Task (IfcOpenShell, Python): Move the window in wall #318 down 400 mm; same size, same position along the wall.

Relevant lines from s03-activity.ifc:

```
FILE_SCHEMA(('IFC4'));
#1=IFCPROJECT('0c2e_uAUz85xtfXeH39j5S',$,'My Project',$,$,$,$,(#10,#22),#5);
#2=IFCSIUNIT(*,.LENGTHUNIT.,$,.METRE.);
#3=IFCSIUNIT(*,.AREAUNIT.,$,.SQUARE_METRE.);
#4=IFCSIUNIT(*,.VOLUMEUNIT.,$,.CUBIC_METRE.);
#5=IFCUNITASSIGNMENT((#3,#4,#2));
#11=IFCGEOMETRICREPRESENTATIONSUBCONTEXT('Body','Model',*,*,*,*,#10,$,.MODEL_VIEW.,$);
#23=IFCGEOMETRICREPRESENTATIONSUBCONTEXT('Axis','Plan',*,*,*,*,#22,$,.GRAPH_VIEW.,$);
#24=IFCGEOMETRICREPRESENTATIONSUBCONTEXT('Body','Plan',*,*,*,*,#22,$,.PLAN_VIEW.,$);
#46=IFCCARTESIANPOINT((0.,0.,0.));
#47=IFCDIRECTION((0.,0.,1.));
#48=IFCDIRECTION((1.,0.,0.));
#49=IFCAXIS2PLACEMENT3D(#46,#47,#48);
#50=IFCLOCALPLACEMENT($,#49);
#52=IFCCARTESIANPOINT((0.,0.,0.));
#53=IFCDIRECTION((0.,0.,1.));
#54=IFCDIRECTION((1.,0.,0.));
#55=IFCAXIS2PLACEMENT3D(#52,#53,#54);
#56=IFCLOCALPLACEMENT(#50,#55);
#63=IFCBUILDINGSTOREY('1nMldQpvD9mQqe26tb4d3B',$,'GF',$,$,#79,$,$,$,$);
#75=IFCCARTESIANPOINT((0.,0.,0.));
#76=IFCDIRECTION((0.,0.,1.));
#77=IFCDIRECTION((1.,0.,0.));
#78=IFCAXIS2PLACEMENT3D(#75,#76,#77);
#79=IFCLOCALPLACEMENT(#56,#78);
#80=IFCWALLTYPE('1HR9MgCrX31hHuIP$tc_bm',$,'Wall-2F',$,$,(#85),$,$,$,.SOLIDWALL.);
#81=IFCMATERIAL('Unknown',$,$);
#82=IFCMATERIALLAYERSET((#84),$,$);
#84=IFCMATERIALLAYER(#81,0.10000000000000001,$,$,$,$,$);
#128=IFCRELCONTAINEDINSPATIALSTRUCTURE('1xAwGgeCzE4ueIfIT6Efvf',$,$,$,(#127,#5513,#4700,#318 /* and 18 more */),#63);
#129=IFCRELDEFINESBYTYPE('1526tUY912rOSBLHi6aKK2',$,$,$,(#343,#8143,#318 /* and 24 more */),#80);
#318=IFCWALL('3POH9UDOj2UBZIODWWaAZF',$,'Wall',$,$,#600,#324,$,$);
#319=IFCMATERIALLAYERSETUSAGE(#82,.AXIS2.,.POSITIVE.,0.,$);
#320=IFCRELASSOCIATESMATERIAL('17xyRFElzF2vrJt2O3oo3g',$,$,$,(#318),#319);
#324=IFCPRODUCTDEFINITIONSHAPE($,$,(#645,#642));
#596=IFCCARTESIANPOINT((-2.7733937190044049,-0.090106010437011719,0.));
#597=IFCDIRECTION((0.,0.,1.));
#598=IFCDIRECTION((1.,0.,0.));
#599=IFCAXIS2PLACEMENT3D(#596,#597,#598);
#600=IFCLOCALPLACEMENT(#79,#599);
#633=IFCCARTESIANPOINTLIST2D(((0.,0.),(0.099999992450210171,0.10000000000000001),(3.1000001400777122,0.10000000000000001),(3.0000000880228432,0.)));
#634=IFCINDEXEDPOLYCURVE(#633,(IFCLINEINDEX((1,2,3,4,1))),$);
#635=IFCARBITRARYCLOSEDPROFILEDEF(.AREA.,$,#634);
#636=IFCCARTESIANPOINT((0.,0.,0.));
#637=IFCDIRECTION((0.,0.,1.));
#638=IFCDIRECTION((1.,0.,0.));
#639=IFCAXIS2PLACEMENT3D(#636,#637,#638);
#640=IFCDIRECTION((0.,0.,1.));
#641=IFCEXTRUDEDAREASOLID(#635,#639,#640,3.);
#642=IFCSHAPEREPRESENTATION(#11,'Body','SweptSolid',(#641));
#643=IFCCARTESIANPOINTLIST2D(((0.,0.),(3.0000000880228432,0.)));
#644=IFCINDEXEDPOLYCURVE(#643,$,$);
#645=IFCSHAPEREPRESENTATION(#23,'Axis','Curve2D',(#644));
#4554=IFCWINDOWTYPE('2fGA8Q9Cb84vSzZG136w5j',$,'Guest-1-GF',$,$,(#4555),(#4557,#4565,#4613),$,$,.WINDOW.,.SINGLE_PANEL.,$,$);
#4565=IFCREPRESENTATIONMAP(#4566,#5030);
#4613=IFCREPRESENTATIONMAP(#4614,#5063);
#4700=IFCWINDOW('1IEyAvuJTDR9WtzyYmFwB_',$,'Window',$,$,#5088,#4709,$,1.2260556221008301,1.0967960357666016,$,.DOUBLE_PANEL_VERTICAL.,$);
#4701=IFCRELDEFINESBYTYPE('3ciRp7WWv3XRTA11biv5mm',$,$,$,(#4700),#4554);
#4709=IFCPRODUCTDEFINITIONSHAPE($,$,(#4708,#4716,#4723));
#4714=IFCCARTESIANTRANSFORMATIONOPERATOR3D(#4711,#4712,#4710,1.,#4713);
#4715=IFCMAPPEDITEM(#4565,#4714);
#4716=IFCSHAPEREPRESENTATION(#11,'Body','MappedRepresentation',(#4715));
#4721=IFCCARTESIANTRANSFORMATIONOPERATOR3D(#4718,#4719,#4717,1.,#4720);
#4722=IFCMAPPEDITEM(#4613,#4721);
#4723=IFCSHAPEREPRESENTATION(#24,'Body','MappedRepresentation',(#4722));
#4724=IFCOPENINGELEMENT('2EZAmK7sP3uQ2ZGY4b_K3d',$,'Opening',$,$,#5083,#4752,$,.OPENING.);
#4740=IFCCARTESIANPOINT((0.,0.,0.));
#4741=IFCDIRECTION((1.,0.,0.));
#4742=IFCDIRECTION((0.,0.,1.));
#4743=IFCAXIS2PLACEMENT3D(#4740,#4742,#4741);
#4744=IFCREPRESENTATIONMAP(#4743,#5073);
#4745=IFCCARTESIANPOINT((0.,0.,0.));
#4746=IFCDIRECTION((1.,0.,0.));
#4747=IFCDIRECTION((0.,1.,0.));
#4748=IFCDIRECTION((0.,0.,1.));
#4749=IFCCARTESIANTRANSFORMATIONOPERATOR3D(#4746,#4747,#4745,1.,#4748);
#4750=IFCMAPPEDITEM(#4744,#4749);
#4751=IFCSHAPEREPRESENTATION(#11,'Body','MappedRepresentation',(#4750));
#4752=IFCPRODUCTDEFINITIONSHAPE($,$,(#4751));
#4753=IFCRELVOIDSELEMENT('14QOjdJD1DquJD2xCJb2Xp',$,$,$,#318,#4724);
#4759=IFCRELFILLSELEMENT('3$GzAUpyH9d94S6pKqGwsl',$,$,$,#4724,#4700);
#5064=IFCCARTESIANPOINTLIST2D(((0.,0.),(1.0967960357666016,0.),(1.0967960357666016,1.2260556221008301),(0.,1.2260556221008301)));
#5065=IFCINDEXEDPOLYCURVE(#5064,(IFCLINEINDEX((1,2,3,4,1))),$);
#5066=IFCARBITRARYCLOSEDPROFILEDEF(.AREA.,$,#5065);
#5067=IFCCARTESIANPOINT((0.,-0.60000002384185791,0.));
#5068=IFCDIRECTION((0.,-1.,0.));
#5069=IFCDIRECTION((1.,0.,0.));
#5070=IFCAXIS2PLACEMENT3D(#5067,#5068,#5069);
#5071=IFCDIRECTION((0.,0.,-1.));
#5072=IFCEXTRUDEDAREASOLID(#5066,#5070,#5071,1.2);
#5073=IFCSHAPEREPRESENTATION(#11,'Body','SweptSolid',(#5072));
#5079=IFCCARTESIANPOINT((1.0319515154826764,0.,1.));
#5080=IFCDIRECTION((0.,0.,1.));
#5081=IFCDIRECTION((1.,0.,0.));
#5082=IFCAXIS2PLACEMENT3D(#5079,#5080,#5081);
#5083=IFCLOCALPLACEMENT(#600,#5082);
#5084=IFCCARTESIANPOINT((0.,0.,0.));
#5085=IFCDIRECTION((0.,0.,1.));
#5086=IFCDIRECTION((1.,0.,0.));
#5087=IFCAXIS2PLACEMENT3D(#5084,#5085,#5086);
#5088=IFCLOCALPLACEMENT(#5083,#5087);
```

```python
import numpy as np
import ifcopenshell
import ifcopenshell.api.geometry
import ifcopenshell.util.placement
import ifcopenshell.util.unit

model = ifcopenshell.open("s03-activity.ifc")
unit_scale = ifcopenshell.util.unit.calculate_unit_scale(model)

window = model.by_id(4700)
opening = window.FillsVoids[0].RelatingOpeningElement
dz = -0.4

shift = np.array([0.0, 0.0, dz])
# The window is placed relative to its opening, so it follows when the opening moves.
matrix = ifcopenshell.util.placement.get_local_placement(opening.ObjectPlacement)
matrix[:3, 3] += shift
ifcopenshell.api.geometry.edit_object_placement(
    model, product=opening, matrix=matrix, is_si=False, should_transform_children=True
)

print(f"moved by {dz * unit_scale:+.3f} m")

model.write("s03-activity-out.ifc")
```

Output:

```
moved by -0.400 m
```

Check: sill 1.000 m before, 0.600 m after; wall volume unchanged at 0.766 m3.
